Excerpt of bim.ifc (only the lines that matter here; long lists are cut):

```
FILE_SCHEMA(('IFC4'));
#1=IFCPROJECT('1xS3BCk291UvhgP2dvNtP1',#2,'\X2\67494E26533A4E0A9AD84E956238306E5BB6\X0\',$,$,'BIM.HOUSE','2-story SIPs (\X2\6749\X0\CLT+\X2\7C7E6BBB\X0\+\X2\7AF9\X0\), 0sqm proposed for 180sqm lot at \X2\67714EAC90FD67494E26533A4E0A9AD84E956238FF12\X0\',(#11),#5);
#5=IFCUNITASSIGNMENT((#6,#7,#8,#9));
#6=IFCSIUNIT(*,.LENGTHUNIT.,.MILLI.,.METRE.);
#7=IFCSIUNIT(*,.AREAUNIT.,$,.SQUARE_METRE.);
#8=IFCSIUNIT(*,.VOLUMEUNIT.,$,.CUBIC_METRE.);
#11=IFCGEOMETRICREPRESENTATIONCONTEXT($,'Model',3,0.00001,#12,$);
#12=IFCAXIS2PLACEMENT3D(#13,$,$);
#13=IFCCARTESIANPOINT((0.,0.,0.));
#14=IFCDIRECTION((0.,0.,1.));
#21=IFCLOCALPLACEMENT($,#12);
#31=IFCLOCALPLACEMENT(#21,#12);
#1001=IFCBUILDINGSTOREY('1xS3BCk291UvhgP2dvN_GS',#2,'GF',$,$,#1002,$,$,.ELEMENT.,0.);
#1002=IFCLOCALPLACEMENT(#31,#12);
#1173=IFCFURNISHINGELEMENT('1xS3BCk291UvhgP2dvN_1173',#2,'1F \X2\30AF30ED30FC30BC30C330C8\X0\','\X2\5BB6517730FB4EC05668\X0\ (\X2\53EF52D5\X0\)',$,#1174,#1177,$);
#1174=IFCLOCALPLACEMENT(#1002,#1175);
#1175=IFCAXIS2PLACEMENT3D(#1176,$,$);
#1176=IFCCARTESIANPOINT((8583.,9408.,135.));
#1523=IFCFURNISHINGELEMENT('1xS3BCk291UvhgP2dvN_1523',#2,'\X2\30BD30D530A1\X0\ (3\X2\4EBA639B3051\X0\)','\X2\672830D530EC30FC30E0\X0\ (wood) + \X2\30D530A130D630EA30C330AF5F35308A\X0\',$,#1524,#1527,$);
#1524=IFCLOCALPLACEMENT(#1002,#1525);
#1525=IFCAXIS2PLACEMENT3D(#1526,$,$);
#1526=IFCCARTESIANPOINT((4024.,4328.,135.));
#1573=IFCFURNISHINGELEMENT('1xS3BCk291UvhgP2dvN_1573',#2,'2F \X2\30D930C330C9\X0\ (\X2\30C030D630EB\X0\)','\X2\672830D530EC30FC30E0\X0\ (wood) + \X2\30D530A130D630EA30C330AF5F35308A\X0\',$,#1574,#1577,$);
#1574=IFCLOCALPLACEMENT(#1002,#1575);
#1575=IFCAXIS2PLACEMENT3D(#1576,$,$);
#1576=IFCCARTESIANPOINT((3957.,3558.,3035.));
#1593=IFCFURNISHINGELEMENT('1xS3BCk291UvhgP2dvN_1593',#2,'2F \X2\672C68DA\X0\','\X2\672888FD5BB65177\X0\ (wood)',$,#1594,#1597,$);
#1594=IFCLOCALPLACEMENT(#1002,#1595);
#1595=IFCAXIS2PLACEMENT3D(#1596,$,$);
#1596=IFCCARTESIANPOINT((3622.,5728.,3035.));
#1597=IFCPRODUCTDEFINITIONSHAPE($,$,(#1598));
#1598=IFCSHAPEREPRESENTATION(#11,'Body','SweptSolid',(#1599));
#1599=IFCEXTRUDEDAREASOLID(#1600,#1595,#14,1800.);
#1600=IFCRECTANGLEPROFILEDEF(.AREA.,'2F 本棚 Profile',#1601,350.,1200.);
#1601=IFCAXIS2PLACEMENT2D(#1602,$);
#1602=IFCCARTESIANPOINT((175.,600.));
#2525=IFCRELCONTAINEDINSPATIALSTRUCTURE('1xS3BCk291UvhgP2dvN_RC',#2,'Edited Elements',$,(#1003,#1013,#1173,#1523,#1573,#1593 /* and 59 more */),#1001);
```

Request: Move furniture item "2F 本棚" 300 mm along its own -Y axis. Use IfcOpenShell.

```python
import ifcopenshell
import ifcopenshell.api.geometry
import ifcopenshell.util.placement
import ifcopenshell.util.unit

model = ifcopenshell.open("bim.ifc")
unit_scale = ifcopenshell.util.unit.calculate_unit_scale(model)

item = model.by_guid("1xS3BCk291UvhgP2dvN_1593")
matrix = ifcopenshell.util.placement.get_local_placement(item.ObjectPlacement)
matrix[:3, 3] -= matrix[:3, 1] * 0.3 / unit_scale
ifcopenshell.api.geometry.edit_object_placement(model, product=item, matrix=matrix, is_si=False)

print(ifcopenshell.util.placement.get_local_placement(item.ObjectPlacement).round(3) + 0.0)

model.write("bim_rev.ifc")
```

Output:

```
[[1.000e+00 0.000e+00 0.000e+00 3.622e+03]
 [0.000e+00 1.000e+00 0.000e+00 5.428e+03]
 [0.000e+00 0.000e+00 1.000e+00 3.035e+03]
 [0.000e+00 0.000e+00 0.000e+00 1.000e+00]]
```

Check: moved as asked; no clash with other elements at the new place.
